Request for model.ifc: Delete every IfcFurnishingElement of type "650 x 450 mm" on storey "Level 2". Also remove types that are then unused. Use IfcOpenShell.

First a look at what the model holds.

```python
import ifcopenshell
import ifcopenshell.util.element

model = ifcopenshell.open("model.ifc")
print(model.schema)
storey = next(s for s in model.by_type("IfcBuildingStorey") if s.Name == "Level 2")
furniture = [e for e in ifcopenshell.util.element.get_decomposition(storey) if e.is_a("IfcFurnishingElement")]
seen = {}
for e in furniture:
    element_type = ifcopenshell.util.element.get_type(e)
    name = element_type.Name if element_type not in (None, e) else None
    seen[name] = seen.get(name, 0) + 1
for name, count in sorted(seen.items(), key=str):
    print(count, "x", name)
```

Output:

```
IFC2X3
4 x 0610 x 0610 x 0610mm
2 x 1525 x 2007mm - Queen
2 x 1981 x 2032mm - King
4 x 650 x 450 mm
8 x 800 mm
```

```python
import ifcopenshell
import ifcopenshell.api.root
import ifcopenshell.util.element

model = ifcopenshell.open("model.ifc")

storey = next(s for s in model.by_type("IfcBuildingStorey") if s.Name == "Level 2")
furniture = [e for e in ifcopenshell.util.element.get_decomposition(storey) if e.is_a("IfcFurnishingElement")]
targets = [e for e in furniture if (t := ifcopenshell.util.element.get_type(e)) not in (None, e) and t.Name == "650 x 450 mm"]
types = {ifcopenshell.util.element.get_type(e) for e in targets} - {None, *targets}

for e in targets:
    ifcopenshell.api.root.remove_product(model, product=e)
print(len(targets), "removed")

unused = [t for t in types if not ifcopenshell.util.element.get_types(t)]
for t in unused:
    ifcopenshell.api.root.remove_product(model, product=t)
print(len(unused), "unused types removed")

model.write("model_v2.ifc")
```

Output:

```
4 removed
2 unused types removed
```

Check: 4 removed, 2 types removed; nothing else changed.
